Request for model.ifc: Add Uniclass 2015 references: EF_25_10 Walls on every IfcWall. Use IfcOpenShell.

First a look at what the model holds.

```python
import ifcopenshell

model = ifcopenshell.open("model.ifc")
print(model.schema)
print("classifications:", [c.Name for c in model.by_type("IfcClassification")])
for ifc_class in ("IfcDoor", "IfcRoof", "IfcStair", "IfcWall", "IfcWindow"):
    print(ifc_class, len(model.by_type(ifc_class)))
```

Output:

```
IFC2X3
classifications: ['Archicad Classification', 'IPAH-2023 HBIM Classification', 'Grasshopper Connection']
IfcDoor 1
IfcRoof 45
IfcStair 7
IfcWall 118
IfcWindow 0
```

```python
import ifcopenshell
import ifcopenshell.api.classification

model = ifcopenshell.open("model.ifc")

# IFC2X3 requires Source and Edition and has no link from the project to the system.
system = model.create_entity("IfcClassification", Source="NBS", Edition="2015", Name="Uniclass 2015")

codes = {
    "IfcWall": ("EF_25_10", "Walls"),
}
for ifc_class, (code, name) in codes.items():
    products = model.by_type(ifc_class)
    ifcopenshell.api.classification.add_reference(
        model, products=products, classification=system, identification=code, name=name
    )
    print(code, len(products))

model.write("model-out.ifc")
```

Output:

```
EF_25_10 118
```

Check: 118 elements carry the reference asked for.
